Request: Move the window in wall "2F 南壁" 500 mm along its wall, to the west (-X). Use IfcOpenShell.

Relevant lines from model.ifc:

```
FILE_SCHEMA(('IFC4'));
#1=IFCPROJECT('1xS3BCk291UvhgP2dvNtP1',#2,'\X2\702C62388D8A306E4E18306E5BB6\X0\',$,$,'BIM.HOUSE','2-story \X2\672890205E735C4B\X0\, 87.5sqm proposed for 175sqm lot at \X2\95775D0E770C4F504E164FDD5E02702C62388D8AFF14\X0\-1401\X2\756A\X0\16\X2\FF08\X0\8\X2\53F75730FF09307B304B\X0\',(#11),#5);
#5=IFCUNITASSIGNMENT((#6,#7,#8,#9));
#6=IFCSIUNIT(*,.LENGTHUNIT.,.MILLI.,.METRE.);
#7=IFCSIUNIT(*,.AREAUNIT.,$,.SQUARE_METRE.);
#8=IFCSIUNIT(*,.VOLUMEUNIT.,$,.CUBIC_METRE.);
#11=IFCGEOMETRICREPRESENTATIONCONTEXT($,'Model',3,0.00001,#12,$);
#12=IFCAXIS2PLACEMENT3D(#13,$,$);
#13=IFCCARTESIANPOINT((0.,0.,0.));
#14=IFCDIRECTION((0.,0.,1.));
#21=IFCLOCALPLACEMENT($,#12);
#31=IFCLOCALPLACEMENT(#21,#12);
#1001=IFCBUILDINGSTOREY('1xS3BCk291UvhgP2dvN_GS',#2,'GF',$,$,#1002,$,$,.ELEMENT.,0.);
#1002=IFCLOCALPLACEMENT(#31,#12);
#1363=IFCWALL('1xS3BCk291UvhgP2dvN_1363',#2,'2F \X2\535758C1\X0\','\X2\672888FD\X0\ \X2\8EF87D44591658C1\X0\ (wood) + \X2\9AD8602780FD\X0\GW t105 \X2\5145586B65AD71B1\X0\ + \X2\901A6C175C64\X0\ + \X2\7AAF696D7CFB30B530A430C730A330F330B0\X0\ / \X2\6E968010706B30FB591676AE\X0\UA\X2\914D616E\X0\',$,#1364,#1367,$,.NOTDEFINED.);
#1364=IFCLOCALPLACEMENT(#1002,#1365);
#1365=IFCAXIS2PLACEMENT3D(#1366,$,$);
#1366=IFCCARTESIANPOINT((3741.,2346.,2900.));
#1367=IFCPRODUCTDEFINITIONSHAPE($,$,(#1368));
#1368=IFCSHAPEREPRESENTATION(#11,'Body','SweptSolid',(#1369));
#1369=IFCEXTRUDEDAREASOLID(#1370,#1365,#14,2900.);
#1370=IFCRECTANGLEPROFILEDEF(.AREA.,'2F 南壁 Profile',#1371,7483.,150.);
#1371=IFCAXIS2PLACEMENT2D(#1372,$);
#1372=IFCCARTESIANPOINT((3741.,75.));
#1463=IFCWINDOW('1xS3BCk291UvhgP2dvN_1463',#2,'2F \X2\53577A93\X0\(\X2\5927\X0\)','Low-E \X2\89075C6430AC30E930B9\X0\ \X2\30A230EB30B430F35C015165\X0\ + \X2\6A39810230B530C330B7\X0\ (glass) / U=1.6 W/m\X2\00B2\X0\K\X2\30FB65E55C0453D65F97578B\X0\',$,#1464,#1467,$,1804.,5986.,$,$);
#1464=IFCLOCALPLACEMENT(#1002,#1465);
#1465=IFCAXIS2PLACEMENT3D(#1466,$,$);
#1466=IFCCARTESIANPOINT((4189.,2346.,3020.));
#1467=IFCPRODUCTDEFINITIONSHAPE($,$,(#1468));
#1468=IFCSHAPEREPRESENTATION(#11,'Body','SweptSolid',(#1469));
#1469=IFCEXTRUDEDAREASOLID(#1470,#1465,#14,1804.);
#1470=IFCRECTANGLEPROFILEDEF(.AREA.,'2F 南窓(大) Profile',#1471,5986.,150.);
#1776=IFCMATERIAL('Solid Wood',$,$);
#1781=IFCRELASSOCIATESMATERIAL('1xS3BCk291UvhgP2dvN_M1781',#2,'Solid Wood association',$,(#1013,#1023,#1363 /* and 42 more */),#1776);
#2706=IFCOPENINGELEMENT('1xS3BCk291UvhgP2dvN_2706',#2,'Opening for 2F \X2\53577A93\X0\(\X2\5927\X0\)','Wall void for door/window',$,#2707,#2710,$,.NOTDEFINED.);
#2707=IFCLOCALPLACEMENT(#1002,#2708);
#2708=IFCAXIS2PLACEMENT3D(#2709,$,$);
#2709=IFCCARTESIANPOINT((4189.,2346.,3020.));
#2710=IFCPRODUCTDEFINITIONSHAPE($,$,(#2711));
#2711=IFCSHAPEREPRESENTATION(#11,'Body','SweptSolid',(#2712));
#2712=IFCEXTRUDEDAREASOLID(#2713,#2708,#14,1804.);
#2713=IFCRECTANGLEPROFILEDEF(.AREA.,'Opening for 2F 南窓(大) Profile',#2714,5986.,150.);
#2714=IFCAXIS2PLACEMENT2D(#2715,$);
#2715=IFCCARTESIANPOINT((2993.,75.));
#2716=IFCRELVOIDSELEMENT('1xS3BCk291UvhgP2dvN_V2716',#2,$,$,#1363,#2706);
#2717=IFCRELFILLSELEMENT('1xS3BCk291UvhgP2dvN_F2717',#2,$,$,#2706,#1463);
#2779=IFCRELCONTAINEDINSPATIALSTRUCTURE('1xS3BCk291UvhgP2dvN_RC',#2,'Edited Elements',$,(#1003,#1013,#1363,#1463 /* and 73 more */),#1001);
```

```python
import ifcopenshell
import ifcopenshell.api.geometry
import ifcopenshell.util.placement

model = ifcopenshell.open("model.ifc")

window = model.by_id(1463)
opening = window.FillsVoids[0].RelatingOpeningElement
wall = opening.VoidsElements[0].RelatingBuildingElement

wall_matrix = ifcopenshell.util.placement.get_local_placement(wall.ObjectPlacement)
shift = wall_matrix[:3, 0] * -500.0
before = ifcopenshell.util.placement.get_local_placement(window.ObjectPlacement)[:3, 3].copy()

# The window is not placed relative to its opening, so move both.
for product in (opening, window):
    matrix = ifcopenshell.util.placement.get_local_placement(product.ObjectPlacement)
    matrix[:3, 3] += shift
    ifcopenshell.api.geometry.edit_object_placement(model, product=product, matrix=matrix, is_si=False)

after = ifcopenshell.util.placement.get_local_placement(window.ObjectPlacement)[:3, 3]
print("window moved by", (after - before).round(3) + 0.0)

model.write("model_rev.ifc")
```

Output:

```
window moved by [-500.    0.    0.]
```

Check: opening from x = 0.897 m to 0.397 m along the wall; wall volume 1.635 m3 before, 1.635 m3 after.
